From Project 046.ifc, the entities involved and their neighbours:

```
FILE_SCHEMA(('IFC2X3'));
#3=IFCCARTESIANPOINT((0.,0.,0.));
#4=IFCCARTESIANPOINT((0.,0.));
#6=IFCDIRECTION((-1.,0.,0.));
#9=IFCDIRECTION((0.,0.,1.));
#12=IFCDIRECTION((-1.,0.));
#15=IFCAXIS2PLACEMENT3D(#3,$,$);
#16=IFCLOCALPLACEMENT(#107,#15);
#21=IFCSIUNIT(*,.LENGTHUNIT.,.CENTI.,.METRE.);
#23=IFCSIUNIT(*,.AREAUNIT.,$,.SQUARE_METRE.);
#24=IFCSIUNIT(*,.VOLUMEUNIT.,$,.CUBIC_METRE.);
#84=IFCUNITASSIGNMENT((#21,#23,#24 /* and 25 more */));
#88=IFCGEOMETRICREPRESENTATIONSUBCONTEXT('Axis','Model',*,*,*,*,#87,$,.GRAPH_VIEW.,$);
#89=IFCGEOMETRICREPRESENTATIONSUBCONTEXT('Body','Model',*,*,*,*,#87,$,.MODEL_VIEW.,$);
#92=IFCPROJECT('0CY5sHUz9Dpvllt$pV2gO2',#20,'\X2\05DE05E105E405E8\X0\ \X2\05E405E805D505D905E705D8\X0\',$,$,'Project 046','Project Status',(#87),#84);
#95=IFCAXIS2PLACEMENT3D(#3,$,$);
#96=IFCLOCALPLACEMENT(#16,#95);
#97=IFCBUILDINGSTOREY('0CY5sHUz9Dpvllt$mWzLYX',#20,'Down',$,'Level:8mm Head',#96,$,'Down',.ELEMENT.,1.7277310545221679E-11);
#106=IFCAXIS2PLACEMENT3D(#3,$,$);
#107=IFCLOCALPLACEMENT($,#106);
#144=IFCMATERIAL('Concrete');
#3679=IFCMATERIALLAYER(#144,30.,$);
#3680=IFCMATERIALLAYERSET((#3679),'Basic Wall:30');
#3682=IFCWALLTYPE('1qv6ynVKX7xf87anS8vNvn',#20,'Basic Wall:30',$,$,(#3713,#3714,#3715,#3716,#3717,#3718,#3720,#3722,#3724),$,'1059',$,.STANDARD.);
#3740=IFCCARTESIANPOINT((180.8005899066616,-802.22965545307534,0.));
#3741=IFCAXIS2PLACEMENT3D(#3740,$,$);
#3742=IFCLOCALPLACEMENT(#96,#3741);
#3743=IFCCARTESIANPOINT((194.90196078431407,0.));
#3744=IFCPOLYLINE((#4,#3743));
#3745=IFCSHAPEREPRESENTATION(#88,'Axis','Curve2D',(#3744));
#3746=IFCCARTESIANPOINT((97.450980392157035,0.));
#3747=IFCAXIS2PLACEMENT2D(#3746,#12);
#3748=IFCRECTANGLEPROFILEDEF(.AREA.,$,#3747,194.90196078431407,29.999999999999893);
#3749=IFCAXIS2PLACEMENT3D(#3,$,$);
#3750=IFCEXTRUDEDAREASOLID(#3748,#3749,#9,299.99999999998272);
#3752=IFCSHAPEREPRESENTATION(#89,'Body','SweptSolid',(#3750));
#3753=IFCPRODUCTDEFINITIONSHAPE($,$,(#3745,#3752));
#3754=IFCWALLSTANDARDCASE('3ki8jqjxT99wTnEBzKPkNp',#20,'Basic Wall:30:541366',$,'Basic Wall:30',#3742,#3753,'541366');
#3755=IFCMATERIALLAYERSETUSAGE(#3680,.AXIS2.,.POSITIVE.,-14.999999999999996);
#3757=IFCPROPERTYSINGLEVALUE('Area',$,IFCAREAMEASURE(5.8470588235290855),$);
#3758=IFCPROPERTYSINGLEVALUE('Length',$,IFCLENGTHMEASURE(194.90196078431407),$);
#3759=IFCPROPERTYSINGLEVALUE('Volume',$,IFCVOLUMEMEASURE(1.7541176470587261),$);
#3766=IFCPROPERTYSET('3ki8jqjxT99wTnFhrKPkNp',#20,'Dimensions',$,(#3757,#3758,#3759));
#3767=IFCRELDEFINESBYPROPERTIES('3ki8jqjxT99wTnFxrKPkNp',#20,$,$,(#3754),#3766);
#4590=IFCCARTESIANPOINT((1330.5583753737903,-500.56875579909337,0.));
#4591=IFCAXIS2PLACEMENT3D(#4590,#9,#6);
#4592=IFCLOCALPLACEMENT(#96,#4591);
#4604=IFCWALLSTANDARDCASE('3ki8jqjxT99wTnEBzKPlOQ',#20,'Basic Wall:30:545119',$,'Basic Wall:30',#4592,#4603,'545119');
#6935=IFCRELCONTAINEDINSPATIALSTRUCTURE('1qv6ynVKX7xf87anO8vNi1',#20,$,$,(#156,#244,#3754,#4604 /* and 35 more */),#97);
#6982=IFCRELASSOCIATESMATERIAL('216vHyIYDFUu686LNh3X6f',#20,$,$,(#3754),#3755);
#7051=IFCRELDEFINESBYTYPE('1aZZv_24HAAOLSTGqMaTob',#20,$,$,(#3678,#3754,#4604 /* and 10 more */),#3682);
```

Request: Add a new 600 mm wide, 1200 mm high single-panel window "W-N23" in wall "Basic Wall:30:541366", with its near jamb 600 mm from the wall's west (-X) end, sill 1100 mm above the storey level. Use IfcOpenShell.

```python
import numpy as np
import ifcopenshell
import ifcopenshell.api.feature
import ifcopenshell.api.geometry
import ifcopenshell.api.pset
import ifcopenshell.api.root
import ifcopenshell.api.spatial
import ifcopenshell.api.type
import ifcopenshell.geom
import ifcopenshell.util.element
import ifcopenshell.util.placement
import ifcopenshell.util.representation
import ifcopenshell.util.shape
import ifcopenshell.util.unit

model = ifcopenshell.open("Project 046.ifc")
unit_scale = ifcopenshell.util.unit.calculate_unit_scale(model)
area_scale = ifcopenshell.util.unit.calculate_unit_scale(model, "AREAUNIT")
volume_scale = ifcopenshell.util.unit.calculate_unit_scale(model, "VOLUMEUNIT")
settings = ifcopenshell.geom.settings()


def volume(element):
    """Net volume in cubic metres, openings subtracted."""
    shape = ifcopenshell.geom.create_shape(settings, element)
    return ifcopenshell.util.shape.get_volume(shape.geometry)


wall = model.by_guid("3ki8jqjxT99wTnEBzKPkNp")
storey = ifcopenshell.util.element.get_container(wall, ifc_class="IfcBuildingStorey")
context = ifcopenshell.util.representation.get_context(model, "Model", "Body", "MODEL_VIEW")
before = volume(wall)

width, height, from_end, sill = 0.6, 1.2, 0.6, 1.1  # metres

# The wall runs along its own X axis, and the end named is its -X end.
wall_shape = ifcopenshell.geom.create_shape(settings, wall)
x, y, z = ifcopenshell.util.shape.get_vertices(wall_shape.geometry).T
start = x.min() + from_end
face, thickness = float(y.min()), float(y.max() - y.min())
wall_matrix = ifcopenshell.util.placement.get_local_placement(wall.ObjectPlacement)
level = ifcopenshell.util.placement.get_local_placement(storey.ObjectPlacement)[2, 3]


def in_wall(x, y):
    """Placement at x, y metres in the wall's axes, at sill height."""
    matrix = wall_matrix.copy()
    matrix[:, 3] = wall_matrix @ np.array([x / unit_scale, y / unit_scale, 0.0, 1.0])
    matrix[2, 3] = level + sill / unit_scale
    return matrix


# Opening: a box that overshoots both wall faces by 50 mm.
opening = ifcopenshell.api.root.create_entity(model, ifc_class="IfcOpeningElement")
box = ifcopenshell.api.geometry.add_wall_representation(
    model, context=context, length=width, height=height, thickness=thickness + 0.1
)
ifcopenshell.api.geometry.assign_representation(model, product=opening, representation=box)
ifcopenshell.api.geometry.edit_object_placement(model, product=opening, matrix=in_wall(start, face - 0.05), is_si=False)
ifcopenshell.api.feature.add_feature(model, feature=opening, element=wall)

window = ifcopenshell.api.root.create_entity(model, ifc_class="IfcWindow", name="W-N23")
window.OverallWidth, window.OverallHeight = width / unit_scale, height / unit_scale
body = ifcopenshell.api.geometry.add_window_representation(
    model,
    context=context,
    overall_width=window.OverallWidth,
    overall_height=window.OverallHeight,
    partition_type="SINGLE_PANEL",
)
ifcopenshell.api.geometry.assign_representation(model, product=window, representation=body)
ifcopenshell.api.spatial.assign_container(model, products=[window], relating_structure=storey)
fills = ifcopenshell.api.feature.add_filling(model, opening=opening, element=window)
fills.OwnerHistory = window.OwnerHistory  # required in IFC2X3

# IFC2X3 keeps the operation on the window style.
style = ifcopenshell.api.root.create_entity(model, ifc_class="IfcWindowStyle", name="W-N23")
style.OperationType, style.ConstructionType = "SINGLE_PANEL", "NOTDEFINED"
style.ParameterTakesPrecedence = style.Sizeable = False
ifcopenshell.api.type.assign_type(model, related_objects=[window], relating_type=style)

# Centre the window in the wall's thickness.
ifcopenshell.api.geometry.edit_object_placement(model, product=window, matrix=in_wall(start, face), is_si=False)
window_shape = ifcopenshell.geom.create_shape(settings, window)
depth = ifcopenshell.util.shape.get_vertices(window_shape.geometry)[:, 1]
offset = face + thickness / 2 - (depth.min() + depth.max()) / 2
ifcopenshell.api.geometry.edit_object_placement(model, product=window, matrix=in_wall(start, offset), is_si=False)

after = volume(wall)

# Update the wall's stored quantities.
pset = model.by_id(ifcopenshell.util.element.get_pset(wall, "Dimensions", should_inherit=False)["id"])
ifcopenshell.api.pset.edit_pset(model, pset=pset, properties={
    "Area": model.create_entity("IfcAreaMeasure", after / thickness / area_scale),
    "Volume": model.create_entity("IfcVolumeMeasure", after / volume_scale),
})

print(f"wall volume {before:.3f} -> {after:.3f} m3")

model.write("Project 046_updated.ifc")
```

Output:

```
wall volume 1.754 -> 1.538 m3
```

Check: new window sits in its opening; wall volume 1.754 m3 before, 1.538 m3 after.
